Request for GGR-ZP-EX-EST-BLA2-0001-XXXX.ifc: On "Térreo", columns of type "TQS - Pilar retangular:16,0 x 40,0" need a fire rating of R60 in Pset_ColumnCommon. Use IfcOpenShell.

First a look at what the model holds.

```python
import ifcopenshell
import ifcopenshell.util.element

model = ifcopenshell.open("GGR-ZP-EX-EST-BLA2-0001-XXXX.ifc")
print(model.schema)
storey = next(s for s in model.by_type("IfcBuildingStorey") if s.Name == "Térreo")
columns = [e for e in ifcopenshell.util.element.get_decomposition(storey) if e.is_a("IfcColumn")]
seen = {}
for e in columns:
    element_type = ifcopenshell.util.element.get_type(e)
    key = (element_type.Name if element_type != e and element_type else None, ifcopenshell.util.element.get_pset(e, "Pset_ColumnCommon", "FireRating"))
    seen[key] = seen.get(key, 0) + 1
for (name, value), count in sorted(seen.items(), key=str):
    print(count, "x", name, "|", value)
```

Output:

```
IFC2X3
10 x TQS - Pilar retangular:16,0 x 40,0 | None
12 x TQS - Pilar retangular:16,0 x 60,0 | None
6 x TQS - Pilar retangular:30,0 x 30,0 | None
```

```python
import ifcopenshell
import ifcopenshell.api.pset
import ifcopenshell.util.element

model = ifcopenshell.open("GGR-ZP-EX-EST-BLA2-0001-XXXX.ifc")

storey = next(s for s in model.by_type("IfcBuildingStorey") if s.Name == "Térreo")
columns = [e for e in ifcopenshell.util.element.get_decomposition(storey) if e.is_a("IfcColumn")]

count = 0
for e in columns:
    element_type = ifcopenshell.util.element.get_type(e)
    if element_type in (None, e) or element_type.Name != "TQS - Pilar retangular:16,0 x 40,0":
        continue
    # add_pset returns the element's existing set when there is one.
    pset = ifcopenshell.api.pset.add_pset(model, product=e, name="Pset_ColumnCommon")
    ifcopenshell.api.pset.edit_pset(model, pset=pset, properties={"FireRating": "R60"})
    count += 1

print(count, "columns updated")

model.write("GGR-ZP-EX-EST-BLA2-0001-XXXX_edited.ifc")
```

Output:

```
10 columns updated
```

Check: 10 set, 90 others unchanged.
